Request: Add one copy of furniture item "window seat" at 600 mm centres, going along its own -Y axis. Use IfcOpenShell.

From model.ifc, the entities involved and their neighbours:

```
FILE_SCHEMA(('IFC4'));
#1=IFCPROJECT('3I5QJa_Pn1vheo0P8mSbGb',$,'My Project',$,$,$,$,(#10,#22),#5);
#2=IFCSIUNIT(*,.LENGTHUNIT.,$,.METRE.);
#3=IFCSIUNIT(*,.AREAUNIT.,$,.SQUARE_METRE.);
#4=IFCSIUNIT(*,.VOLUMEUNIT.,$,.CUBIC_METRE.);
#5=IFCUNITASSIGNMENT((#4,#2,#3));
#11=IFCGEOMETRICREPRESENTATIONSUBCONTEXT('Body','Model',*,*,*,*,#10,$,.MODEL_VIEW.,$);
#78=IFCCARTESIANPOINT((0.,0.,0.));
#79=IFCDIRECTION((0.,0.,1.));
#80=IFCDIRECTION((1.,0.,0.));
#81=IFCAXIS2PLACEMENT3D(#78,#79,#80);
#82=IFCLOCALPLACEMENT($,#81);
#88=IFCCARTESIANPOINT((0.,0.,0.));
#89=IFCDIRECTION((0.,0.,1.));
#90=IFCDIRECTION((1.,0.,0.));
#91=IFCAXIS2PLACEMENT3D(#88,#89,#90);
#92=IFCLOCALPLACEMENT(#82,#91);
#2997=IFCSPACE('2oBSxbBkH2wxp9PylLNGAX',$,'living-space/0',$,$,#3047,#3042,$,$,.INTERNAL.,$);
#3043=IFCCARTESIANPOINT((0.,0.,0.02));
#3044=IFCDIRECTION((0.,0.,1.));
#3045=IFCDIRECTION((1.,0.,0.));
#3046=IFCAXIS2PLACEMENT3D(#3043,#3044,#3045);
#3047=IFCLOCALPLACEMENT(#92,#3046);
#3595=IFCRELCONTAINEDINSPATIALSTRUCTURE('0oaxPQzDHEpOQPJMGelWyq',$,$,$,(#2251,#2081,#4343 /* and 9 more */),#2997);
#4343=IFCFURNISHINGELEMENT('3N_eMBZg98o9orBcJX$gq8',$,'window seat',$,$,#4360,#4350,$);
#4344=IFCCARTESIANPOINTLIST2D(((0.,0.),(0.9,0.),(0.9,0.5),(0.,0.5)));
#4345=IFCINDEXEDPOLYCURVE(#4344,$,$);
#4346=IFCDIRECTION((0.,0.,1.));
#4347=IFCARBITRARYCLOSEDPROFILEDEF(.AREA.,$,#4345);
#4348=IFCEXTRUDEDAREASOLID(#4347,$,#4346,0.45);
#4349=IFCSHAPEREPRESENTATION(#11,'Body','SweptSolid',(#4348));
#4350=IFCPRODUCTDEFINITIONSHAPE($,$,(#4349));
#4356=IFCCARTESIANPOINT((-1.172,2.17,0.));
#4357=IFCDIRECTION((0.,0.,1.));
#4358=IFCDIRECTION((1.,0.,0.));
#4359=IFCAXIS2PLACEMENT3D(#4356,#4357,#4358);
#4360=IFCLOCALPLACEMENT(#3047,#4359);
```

```python
import ifcopenshell
import ifcopenshell.api.geometry
import ifcopenshell.api.root
import ifcopenshell.util.element
import ifcopenshell.util.placement
import ifcopenshell.util.unit

model = ifcopenshell.open("model.ifc")
unit_scale = ifcopenshell.util.unit.calculate_unit_scale(model)

source = model.by_guid("3N_eMBZg98o9orBcJX$gq8")
base = ifcopenshell.util.placement.get_local_placement(source.ObjectPlacement)
step = -base[:3, 1] * 0.6 / unit_scale

for i in range(1, 2):
    copy = ifcopenshell.api.root.copy_class(model, product=source)
    copy.Representation = ifcopenshell.util.element.copy_deep(
        model, source.Representation, exclude=["IfcGeometricRepresentationContext", "IfcRepresentationMap"]
    )
    matrix = base.copy()
    matrix[:3, 3] += i * step
    print("added at", matrix[:3, 3].round(3) + 0.0)
    ifcopenshell.api.geometry.edit_object_placement(model, product=copy, matrix=matrix, is_si=False)

model.write("model_updated.ifc")
```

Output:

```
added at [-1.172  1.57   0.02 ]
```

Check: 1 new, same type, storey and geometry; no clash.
